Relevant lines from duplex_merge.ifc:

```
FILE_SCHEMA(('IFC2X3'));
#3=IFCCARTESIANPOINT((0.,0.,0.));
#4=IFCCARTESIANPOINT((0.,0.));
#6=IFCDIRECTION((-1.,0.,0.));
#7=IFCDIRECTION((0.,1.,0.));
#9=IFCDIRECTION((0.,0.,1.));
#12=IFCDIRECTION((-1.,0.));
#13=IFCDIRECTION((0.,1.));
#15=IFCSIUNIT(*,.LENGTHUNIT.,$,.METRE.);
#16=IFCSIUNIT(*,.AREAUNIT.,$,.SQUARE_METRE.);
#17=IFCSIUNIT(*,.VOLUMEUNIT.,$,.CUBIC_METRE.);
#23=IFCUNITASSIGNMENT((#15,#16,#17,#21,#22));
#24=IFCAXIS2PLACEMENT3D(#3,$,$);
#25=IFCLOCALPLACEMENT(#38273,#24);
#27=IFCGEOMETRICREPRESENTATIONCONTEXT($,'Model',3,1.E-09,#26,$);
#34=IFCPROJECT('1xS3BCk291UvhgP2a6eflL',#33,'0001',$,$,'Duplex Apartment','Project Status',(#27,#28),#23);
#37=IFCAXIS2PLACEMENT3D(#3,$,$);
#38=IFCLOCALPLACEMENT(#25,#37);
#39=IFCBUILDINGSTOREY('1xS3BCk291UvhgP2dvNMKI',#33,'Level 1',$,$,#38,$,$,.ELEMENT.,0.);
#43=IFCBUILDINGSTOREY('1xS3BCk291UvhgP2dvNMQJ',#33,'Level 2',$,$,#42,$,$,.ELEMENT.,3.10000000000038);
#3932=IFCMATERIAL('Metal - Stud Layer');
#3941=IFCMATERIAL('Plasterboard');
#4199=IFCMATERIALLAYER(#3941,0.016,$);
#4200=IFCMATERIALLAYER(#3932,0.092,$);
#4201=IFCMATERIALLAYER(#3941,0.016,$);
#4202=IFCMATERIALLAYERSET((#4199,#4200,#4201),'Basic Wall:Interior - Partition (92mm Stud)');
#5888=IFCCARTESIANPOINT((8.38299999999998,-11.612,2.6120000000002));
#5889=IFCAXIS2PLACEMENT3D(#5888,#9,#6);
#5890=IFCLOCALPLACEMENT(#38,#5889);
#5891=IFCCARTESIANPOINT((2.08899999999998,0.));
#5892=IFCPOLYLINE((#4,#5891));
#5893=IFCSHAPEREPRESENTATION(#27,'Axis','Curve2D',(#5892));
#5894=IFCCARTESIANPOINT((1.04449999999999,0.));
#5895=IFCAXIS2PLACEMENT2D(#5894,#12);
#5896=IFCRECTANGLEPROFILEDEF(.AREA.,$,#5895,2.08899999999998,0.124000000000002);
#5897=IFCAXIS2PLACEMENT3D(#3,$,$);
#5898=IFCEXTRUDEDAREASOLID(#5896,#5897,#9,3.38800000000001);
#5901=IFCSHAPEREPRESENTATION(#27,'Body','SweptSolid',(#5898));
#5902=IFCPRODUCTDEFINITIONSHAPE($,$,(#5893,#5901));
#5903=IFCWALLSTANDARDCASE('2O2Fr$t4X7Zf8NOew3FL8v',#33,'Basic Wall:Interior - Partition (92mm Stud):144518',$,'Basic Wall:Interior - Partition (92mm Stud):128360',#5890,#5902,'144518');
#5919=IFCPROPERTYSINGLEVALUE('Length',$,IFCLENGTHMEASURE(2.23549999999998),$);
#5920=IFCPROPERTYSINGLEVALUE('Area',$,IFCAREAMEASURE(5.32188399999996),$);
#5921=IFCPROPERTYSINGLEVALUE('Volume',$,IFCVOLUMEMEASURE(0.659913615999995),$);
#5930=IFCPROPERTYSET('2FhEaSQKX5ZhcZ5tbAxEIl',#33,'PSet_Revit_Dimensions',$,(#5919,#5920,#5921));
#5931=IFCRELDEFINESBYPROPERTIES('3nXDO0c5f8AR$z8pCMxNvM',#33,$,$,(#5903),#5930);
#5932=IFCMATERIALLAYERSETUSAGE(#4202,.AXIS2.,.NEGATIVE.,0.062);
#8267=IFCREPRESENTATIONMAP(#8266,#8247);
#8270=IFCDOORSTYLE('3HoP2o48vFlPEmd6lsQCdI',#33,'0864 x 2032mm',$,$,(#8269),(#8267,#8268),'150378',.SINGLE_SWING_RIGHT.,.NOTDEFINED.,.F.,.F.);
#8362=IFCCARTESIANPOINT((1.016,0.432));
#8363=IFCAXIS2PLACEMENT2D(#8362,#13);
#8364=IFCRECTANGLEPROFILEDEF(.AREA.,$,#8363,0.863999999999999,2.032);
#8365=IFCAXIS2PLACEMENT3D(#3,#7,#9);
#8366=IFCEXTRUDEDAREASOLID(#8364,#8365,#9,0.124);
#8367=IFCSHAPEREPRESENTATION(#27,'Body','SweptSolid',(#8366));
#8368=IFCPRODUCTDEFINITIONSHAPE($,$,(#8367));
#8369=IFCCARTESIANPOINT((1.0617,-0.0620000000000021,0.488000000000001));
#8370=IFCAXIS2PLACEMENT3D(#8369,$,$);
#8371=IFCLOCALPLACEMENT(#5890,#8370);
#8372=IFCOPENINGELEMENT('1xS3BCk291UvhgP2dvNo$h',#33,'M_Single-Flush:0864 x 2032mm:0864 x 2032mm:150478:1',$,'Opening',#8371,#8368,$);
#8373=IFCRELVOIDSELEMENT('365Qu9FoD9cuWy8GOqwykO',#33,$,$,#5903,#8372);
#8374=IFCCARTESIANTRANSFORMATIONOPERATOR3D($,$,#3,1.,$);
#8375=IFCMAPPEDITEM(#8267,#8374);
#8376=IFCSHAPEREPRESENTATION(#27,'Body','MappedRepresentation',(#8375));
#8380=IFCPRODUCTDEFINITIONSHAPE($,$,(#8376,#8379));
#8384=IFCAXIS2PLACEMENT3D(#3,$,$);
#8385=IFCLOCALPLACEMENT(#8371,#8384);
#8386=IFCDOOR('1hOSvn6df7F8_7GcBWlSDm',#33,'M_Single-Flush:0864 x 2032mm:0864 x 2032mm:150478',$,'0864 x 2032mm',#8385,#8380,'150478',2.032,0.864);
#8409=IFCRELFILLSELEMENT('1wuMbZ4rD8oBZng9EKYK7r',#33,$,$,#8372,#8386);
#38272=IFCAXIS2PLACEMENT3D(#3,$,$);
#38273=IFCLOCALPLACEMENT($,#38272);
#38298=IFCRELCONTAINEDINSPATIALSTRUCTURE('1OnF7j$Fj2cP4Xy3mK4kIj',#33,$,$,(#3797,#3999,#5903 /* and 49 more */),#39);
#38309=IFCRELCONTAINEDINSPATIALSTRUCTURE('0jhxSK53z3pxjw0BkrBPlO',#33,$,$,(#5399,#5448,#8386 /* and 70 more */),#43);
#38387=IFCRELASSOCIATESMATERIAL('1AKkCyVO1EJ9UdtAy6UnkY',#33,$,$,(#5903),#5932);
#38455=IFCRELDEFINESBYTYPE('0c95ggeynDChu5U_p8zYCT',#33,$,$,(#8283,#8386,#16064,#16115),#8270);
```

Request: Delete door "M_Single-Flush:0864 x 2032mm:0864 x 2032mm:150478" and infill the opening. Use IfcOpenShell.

```python
import ifcopenshell
import ifcopenshell.api.feature
import ifcopenshell.api.pset
import ifcopenshell.api.root
import ifcopenshell.geom
import ifcopenshell.util.element
import ifcopenshell.util.shape
import ifcopenshell.util.unit

model = ifcopenshell.open("duplex_merge.ifc")
area_scale = ifcopenshell.util.unit.calculate_unit_scale(model, "AREAUNIT")
volume_scale = ifcopenshell.util.unit.calculate_unit_scale(model, "VOLUMEUNIT")
settings = ifcopenshell.geom.settings()


def volume(element):
    """Net volume in cubic metres, openings subtracted."""
    shape = ifcopenshell.geom.create_shape(settings, element)
    return ifcopenshell.util.shape.get_volume(shape.geometry)


door = model.by_id(8386)
opening = door.FillsVoids[0].RelatingOpeningElement
wall = opening.VoidsElements[0].RelatingBuildingElement
before = volume(wall)

ifcopenshell.api.root.remove_product(model, product=door)
ifcopenshell.api.feature.remove_feature(model, feature=opening)

after = volume(wall)
thickness = 0.124  # wall thickness in metres

# Update the wall's stored quantities.
pset = model.by_id(ifcopenshell.util.element.get_pset(wall, "PSet_Revit_Dimensions", should_inherit=False)["id"])
ifcopenshell.api.pset.edit_pset(model, pset=pset, properties={
    "Area": model.create_entity("IfcAreaMeasure", after / thickness / area_scale),
    "Volume": model.create_entity("IfcVolumeMeasure", after / volume_scale),
})

print(f"wall volume {before:.3f} -> {after:.3f} m3")

model.write("duplex_merge_v2.ifc")
```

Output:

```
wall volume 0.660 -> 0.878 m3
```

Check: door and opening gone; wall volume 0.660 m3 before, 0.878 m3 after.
